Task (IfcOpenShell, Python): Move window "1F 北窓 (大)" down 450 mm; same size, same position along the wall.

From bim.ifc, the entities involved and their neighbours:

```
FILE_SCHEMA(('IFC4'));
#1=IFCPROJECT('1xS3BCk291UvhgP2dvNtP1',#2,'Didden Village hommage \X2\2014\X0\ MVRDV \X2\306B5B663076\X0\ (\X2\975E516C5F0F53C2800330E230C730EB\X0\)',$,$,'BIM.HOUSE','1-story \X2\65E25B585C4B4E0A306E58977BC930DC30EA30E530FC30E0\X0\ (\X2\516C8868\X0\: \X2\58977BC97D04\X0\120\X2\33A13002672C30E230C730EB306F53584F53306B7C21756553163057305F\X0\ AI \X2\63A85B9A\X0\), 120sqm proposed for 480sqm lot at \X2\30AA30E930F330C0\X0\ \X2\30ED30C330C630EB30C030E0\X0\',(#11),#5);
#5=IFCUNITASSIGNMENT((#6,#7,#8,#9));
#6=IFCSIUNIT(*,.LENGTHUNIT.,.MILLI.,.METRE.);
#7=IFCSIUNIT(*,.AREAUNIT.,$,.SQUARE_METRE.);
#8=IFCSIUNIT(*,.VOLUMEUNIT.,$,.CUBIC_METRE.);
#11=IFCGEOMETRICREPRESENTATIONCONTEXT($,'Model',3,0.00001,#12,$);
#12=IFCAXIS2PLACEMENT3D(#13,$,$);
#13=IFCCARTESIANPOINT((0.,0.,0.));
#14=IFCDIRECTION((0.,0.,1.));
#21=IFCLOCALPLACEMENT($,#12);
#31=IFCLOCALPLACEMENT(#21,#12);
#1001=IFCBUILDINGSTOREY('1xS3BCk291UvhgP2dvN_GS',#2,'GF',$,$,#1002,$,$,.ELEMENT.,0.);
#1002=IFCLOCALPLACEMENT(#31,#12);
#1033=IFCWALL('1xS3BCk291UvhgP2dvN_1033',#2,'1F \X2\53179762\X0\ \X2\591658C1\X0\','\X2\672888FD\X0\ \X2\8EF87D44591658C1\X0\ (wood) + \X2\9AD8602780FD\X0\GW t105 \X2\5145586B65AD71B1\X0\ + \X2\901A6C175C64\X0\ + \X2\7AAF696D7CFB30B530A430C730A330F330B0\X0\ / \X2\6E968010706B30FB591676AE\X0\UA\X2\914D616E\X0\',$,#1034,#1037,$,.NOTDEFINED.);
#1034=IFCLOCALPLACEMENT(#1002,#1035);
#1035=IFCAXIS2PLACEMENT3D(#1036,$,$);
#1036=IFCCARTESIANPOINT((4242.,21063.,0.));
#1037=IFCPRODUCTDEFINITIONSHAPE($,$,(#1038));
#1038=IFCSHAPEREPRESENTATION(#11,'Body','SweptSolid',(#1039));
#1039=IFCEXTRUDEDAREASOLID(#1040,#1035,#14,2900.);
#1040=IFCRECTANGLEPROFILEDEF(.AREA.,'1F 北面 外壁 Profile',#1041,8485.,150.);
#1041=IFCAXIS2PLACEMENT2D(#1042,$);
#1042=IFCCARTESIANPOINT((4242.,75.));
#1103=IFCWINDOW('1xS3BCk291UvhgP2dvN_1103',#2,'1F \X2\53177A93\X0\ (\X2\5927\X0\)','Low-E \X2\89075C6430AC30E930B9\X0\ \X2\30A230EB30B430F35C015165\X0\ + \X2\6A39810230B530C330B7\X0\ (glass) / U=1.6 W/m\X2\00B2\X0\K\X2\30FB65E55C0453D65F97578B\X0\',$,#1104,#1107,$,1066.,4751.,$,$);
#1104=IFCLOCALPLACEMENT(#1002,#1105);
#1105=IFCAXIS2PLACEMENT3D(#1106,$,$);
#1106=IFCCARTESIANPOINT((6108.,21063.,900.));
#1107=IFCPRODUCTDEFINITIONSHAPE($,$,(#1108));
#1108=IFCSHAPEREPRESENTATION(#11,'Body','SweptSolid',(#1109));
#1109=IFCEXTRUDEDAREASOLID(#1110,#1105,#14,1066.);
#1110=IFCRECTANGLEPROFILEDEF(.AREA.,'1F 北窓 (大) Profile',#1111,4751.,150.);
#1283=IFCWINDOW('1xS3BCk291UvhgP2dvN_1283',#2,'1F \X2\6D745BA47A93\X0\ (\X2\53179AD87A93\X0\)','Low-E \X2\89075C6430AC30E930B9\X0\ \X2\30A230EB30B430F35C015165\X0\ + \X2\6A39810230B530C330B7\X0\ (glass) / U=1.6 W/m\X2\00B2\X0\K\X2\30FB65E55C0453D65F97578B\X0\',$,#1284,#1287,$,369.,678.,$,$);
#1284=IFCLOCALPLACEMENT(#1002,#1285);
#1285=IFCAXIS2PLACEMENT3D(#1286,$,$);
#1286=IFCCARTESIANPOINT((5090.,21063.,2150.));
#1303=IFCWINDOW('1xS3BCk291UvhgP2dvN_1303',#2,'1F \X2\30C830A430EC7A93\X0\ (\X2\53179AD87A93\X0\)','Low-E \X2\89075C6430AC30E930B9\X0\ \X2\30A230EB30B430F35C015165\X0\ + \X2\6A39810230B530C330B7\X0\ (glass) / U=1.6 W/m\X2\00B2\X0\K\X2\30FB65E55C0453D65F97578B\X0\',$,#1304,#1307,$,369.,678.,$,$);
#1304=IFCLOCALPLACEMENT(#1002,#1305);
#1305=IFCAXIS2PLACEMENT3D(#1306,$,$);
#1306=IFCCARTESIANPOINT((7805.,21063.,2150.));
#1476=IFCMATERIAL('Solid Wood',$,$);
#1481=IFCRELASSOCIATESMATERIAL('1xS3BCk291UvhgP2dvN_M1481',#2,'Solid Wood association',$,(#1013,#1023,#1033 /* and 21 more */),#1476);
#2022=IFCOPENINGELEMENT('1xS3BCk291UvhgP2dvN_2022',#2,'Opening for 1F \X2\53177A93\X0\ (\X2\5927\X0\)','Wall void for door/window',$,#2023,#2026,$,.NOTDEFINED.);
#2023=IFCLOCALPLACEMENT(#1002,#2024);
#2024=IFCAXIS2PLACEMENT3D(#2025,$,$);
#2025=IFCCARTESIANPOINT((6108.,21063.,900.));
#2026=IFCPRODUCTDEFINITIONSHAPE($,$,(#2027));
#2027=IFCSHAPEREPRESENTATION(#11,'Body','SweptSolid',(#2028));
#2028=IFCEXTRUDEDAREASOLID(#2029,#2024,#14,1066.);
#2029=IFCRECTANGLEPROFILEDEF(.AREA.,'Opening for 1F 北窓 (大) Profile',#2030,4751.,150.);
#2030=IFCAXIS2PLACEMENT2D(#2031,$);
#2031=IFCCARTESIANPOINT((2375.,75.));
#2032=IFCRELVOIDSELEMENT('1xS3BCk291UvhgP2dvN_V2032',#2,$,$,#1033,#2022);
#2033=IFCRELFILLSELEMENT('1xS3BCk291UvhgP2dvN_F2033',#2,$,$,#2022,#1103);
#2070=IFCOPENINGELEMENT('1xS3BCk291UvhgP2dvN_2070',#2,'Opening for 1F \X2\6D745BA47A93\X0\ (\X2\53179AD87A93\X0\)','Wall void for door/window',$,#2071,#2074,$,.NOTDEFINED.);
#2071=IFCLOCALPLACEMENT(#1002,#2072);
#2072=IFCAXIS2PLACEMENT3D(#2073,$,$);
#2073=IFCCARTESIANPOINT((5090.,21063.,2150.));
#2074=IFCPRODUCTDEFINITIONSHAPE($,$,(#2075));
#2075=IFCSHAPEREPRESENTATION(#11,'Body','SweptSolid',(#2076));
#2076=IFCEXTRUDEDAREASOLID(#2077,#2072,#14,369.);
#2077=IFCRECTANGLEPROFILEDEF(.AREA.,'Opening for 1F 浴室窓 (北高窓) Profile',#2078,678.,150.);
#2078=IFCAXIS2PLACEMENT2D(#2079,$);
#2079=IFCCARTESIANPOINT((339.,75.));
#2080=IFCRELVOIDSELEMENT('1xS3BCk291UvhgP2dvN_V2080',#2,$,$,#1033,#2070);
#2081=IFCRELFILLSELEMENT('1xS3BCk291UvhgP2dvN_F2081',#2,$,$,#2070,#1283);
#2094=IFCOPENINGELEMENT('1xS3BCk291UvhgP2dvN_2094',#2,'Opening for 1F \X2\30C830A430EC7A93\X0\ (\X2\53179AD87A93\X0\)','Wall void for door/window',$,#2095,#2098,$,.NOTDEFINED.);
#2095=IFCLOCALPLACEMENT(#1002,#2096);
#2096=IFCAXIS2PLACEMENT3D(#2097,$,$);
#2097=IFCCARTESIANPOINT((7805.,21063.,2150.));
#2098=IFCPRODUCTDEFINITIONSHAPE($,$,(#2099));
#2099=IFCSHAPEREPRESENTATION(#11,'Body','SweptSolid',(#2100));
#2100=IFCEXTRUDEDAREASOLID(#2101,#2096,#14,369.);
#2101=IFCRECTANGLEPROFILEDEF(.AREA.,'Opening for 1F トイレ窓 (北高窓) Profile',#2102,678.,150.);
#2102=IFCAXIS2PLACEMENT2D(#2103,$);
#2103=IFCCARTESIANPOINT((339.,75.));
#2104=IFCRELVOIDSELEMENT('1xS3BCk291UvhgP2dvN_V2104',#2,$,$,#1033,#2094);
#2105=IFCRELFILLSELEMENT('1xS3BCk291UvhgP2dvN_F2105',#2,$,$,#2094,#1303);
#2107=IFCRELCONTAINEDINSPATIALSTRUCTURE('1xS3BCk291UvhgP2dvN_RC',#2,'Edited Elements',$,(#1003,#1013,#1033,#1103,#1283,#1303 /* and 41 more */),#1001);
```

```python
import numpy as np
import ifcopenshell
import ifcopenshell.api.geometry
import ifcopenshell.util.placement
import ifcopenshell.util.unit

model = ifcopenshell.open("bim.ifc")
unit_scale = ifcopenshell.util.unit.calculate_unit_scale(model)

window = model.by_id(1103)
opening = window.FillsVoids[0].RelatingOpeningElement
dz = -0.45 / unit_scale

shift = np.array([0.0, 0.0, dz])
# The window is not placed relative to its opening, so move both.
for product in (opening, window):
    matrix = ifcopenshell.util.placement.get_local_placement(product.ObjectPlacement)
    matrix[:3, 3] += shift
    ifcopenshell.api.geometry.edit_object_placement(model, product=product, matrix=matrix, is_si=False)

print(f"moved by {dz * unit_scale:+.3f} m")

model.write("bim_rev.ifc")
```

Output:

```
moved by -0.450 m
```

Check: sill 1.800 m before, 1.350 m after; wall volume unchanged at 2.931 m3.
